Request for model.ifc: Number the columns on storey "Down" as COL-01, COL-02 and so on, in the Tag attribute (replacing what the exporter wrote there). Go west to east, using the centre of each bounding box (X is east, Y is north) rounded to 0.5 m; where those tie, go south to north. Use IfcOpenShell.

First a look at what the model holds.

```python
import ifcopenshell
import ifcopenshell.util.element
import ifcopenshell.util.placement

model = ifcopenshell.open("model.ifc")
print(model.schema)
storey = next(s for s in model.by_type("IfcBuildingStorey") if s.Name == "Down")
columns = [e for e in ifcopenshell.util.element.get_decomposition(storey) if e.is_a("IfcColumn")]
for e in sorted(columns, key=lambda e: e.id()):
    origin = ifcopenshell.util.placement.get_local_placement(e.ObjectPlacement)[:3, 3]
    print(e.id(), e.Tag, e.Name, origin.round(2) + 0.0, sep=" | ")
```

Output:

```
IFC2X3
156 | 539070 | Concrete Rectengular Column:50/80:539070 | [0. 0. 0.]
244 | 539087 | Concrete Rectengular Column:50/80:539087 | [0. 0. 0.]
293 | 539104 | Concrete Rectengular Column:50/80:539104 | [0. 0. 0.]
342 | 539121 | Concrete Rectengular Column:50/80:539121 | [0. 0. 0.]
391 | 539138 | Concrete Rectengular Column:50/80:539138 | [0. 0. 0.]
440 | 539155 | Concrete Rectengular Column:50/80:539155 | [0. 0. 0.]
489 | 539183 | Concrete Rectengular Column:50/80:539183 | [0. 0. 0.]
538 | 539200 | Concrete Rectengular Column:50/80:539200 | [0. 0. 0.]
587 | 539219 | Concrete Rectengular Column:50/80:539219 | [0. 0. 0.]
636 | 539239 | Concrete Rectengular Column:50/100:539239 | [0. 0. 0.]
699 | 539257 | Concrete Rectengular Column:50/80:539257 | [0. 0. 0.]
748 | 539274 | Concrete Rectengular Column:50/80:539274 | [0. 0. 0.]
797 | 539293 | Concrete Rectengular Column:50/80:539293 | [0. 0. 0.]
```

```python
import ifcopenshell
import ifcopenshell.geom
import ifcopenshell.util.element
import ifcopenshell.util.shape

model = ifcopenshell.open("model.ifc")
settings = ifcopenshell.geom.settings()
settings.set("use-world-coords", True)


def centre(element):
    shape = ifcopenshell.geom.create_shape(settings, element)
    return ifcopenshell.util.shape.get_bbox_centroid(shape.geometry)


storey = next(s for s in model.by_type("IfcBuildingStorey") if s.Name == "Down")
columns = [e for e in ifcopenshell.util.element.get_decomposition(storey) if e.is_a("IfcColumn")]

# Insertion points can sit at a corner or the storey origin, so sort by the geometry (in metres).
centres = {e: centre(e) for e in columns}
columns.sort(key=lambda e: (round(centres[e][0] / 0.5), centres[e][1]))

for i, e in enumerate(columns, start=1):
    number = f"COL-{i:02d}"
    e.Tag = number
    print(e.id(), number)

model.write("model_updated.ifc")
```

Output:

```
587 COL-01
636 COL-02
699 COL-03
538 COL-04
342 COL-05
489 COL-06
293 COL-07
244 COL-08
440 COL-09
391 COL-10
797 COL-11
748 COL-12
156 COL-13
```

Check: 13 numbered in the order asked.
